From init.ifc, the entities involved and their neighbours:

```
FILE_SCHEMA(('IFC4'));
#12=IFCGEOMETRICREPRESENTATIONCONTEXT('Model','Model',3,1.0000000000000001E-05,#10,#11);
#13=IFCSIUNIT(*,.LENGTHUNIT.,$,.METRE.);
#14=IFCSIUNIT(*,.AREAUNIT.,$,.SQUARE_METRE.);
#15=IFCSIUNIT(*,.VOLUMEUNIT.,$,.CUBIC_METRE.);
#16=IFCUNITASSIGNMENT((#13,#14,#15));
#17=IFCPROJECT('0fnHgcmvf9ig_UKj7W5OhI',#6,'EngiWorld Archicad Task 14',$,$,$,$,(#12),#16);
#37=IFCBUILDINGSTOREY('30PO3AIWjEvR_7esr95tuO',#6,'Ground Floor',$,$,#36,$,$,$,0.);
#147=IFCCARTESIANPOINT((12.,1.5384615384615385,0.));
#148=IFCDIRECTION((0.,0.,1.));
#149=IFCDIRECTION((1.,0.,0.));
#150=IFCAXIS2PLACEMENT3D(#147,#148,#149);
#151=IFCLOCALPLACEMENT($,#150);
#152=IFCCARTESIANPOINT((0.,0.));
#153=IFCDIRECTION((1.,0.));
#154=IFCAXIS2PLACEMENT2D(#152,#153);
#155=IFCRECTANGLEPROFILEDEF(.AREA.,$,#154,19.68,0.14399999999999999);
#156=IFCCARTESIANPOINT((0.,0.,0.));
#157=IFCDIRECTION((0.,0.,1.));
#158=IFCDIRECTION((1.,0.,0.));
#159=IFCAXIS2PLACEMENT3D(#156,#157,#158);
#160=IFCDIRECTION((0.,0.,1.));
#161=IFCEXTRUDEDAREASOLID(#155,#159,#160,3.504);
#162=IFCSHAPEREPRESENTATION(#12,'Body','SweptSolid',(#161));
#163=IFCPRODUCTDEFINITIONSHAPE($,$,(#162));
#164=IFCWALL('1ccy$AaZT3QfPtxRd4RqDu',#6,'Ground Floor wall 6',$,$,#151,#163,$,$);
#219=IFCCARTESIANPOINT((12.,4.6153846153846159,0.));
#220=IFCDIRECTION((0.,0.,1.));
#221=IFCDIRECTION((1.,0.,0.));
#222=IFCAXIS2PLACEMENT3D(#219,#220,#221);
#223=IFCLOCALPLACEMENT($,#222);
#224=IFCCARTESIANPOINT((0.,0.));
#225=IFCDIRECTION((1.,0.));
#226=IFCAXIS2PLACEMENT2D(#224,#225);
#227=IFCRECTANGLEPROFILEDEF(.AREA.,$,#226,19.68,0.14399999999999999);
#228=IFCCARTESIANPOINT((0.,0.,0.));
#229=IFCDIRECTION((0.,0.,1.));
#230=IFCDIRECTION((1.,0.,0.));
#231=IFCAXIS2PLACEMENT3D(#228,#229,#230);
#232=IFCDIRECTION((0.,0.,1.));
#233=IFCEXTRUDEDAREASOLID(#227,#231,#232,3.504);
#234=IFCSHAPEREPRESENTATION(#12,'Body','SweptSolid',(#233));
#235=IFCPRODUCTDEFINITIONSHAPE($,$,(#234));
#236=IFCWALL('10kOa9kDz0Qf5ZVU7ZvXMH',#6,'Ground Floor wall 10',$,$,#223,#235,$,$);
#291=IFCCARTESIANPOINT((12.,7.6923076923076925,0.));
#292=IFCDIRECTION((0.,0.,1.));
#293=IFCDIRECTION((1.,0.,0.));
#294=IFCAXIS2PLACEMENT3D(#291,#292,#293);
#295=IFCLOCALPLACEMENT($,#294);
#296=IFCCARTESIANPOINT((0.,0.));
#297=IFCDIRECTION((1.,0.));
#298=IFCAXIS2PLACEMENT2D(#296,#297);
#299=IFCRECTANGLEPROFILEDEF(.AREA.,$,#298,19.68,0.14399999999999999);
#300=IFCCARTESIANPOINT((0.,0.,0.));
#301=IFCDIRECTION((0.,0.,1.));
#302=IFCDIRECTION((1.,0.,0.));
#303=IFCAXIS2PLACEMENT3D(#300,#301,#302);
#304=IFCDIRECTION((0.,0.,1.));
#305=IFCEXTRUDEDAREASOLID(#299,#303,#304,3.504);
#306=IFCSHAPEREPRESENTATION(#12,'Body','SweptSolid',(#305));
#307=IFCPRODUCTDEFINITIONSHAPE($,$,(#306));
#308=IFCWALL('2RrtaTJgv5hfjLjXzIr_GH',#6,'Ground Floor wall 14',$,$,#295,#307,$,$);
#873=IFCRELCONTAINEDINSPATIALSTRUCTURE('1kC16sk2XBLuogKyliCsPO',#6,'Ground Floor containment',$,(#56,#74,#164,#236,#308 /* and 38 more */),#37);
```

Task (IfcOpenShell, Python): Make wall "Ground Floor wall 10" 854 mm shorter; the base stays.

```python
import ifcopenshell
import ifcopenshell.geom
import ifcopenshell.util.shape
import ifcopenshell.util.unit

model = ifcopenshell.open("init.ifc")
unit_scale = ifcopenshell.util.unit.calculate_unit_scale(model)
settings = ifcopenshell.geom.settings()


def volume(element):
    """Net volume in cubic metres, openings subtracted."""
    shape = ifcopenshell.geom.create_shape(settings, element)
    return ifcopenshell.util.shape.get_volume(shape.geometry)


wall = model.by_id(236)
before = volume(wall)

body = next(r for r in wall.Representation.Representations if r.RepresentationIdentifier == "Body")
solid = body.Items[0]
old_height = solid.Depth
solid.Depth -= 0.854 / unit_scale
after = volume(wall)

print(f"height {old_height:g} -> {solid.Depth:g}, volume {before:.3f} -> {after:.3f} m3")

model.write("init_v2.ifc")
```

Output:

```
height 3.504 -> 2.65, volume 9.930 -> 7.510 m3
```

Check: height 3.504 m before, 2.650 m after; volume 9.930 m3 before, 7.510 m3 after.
